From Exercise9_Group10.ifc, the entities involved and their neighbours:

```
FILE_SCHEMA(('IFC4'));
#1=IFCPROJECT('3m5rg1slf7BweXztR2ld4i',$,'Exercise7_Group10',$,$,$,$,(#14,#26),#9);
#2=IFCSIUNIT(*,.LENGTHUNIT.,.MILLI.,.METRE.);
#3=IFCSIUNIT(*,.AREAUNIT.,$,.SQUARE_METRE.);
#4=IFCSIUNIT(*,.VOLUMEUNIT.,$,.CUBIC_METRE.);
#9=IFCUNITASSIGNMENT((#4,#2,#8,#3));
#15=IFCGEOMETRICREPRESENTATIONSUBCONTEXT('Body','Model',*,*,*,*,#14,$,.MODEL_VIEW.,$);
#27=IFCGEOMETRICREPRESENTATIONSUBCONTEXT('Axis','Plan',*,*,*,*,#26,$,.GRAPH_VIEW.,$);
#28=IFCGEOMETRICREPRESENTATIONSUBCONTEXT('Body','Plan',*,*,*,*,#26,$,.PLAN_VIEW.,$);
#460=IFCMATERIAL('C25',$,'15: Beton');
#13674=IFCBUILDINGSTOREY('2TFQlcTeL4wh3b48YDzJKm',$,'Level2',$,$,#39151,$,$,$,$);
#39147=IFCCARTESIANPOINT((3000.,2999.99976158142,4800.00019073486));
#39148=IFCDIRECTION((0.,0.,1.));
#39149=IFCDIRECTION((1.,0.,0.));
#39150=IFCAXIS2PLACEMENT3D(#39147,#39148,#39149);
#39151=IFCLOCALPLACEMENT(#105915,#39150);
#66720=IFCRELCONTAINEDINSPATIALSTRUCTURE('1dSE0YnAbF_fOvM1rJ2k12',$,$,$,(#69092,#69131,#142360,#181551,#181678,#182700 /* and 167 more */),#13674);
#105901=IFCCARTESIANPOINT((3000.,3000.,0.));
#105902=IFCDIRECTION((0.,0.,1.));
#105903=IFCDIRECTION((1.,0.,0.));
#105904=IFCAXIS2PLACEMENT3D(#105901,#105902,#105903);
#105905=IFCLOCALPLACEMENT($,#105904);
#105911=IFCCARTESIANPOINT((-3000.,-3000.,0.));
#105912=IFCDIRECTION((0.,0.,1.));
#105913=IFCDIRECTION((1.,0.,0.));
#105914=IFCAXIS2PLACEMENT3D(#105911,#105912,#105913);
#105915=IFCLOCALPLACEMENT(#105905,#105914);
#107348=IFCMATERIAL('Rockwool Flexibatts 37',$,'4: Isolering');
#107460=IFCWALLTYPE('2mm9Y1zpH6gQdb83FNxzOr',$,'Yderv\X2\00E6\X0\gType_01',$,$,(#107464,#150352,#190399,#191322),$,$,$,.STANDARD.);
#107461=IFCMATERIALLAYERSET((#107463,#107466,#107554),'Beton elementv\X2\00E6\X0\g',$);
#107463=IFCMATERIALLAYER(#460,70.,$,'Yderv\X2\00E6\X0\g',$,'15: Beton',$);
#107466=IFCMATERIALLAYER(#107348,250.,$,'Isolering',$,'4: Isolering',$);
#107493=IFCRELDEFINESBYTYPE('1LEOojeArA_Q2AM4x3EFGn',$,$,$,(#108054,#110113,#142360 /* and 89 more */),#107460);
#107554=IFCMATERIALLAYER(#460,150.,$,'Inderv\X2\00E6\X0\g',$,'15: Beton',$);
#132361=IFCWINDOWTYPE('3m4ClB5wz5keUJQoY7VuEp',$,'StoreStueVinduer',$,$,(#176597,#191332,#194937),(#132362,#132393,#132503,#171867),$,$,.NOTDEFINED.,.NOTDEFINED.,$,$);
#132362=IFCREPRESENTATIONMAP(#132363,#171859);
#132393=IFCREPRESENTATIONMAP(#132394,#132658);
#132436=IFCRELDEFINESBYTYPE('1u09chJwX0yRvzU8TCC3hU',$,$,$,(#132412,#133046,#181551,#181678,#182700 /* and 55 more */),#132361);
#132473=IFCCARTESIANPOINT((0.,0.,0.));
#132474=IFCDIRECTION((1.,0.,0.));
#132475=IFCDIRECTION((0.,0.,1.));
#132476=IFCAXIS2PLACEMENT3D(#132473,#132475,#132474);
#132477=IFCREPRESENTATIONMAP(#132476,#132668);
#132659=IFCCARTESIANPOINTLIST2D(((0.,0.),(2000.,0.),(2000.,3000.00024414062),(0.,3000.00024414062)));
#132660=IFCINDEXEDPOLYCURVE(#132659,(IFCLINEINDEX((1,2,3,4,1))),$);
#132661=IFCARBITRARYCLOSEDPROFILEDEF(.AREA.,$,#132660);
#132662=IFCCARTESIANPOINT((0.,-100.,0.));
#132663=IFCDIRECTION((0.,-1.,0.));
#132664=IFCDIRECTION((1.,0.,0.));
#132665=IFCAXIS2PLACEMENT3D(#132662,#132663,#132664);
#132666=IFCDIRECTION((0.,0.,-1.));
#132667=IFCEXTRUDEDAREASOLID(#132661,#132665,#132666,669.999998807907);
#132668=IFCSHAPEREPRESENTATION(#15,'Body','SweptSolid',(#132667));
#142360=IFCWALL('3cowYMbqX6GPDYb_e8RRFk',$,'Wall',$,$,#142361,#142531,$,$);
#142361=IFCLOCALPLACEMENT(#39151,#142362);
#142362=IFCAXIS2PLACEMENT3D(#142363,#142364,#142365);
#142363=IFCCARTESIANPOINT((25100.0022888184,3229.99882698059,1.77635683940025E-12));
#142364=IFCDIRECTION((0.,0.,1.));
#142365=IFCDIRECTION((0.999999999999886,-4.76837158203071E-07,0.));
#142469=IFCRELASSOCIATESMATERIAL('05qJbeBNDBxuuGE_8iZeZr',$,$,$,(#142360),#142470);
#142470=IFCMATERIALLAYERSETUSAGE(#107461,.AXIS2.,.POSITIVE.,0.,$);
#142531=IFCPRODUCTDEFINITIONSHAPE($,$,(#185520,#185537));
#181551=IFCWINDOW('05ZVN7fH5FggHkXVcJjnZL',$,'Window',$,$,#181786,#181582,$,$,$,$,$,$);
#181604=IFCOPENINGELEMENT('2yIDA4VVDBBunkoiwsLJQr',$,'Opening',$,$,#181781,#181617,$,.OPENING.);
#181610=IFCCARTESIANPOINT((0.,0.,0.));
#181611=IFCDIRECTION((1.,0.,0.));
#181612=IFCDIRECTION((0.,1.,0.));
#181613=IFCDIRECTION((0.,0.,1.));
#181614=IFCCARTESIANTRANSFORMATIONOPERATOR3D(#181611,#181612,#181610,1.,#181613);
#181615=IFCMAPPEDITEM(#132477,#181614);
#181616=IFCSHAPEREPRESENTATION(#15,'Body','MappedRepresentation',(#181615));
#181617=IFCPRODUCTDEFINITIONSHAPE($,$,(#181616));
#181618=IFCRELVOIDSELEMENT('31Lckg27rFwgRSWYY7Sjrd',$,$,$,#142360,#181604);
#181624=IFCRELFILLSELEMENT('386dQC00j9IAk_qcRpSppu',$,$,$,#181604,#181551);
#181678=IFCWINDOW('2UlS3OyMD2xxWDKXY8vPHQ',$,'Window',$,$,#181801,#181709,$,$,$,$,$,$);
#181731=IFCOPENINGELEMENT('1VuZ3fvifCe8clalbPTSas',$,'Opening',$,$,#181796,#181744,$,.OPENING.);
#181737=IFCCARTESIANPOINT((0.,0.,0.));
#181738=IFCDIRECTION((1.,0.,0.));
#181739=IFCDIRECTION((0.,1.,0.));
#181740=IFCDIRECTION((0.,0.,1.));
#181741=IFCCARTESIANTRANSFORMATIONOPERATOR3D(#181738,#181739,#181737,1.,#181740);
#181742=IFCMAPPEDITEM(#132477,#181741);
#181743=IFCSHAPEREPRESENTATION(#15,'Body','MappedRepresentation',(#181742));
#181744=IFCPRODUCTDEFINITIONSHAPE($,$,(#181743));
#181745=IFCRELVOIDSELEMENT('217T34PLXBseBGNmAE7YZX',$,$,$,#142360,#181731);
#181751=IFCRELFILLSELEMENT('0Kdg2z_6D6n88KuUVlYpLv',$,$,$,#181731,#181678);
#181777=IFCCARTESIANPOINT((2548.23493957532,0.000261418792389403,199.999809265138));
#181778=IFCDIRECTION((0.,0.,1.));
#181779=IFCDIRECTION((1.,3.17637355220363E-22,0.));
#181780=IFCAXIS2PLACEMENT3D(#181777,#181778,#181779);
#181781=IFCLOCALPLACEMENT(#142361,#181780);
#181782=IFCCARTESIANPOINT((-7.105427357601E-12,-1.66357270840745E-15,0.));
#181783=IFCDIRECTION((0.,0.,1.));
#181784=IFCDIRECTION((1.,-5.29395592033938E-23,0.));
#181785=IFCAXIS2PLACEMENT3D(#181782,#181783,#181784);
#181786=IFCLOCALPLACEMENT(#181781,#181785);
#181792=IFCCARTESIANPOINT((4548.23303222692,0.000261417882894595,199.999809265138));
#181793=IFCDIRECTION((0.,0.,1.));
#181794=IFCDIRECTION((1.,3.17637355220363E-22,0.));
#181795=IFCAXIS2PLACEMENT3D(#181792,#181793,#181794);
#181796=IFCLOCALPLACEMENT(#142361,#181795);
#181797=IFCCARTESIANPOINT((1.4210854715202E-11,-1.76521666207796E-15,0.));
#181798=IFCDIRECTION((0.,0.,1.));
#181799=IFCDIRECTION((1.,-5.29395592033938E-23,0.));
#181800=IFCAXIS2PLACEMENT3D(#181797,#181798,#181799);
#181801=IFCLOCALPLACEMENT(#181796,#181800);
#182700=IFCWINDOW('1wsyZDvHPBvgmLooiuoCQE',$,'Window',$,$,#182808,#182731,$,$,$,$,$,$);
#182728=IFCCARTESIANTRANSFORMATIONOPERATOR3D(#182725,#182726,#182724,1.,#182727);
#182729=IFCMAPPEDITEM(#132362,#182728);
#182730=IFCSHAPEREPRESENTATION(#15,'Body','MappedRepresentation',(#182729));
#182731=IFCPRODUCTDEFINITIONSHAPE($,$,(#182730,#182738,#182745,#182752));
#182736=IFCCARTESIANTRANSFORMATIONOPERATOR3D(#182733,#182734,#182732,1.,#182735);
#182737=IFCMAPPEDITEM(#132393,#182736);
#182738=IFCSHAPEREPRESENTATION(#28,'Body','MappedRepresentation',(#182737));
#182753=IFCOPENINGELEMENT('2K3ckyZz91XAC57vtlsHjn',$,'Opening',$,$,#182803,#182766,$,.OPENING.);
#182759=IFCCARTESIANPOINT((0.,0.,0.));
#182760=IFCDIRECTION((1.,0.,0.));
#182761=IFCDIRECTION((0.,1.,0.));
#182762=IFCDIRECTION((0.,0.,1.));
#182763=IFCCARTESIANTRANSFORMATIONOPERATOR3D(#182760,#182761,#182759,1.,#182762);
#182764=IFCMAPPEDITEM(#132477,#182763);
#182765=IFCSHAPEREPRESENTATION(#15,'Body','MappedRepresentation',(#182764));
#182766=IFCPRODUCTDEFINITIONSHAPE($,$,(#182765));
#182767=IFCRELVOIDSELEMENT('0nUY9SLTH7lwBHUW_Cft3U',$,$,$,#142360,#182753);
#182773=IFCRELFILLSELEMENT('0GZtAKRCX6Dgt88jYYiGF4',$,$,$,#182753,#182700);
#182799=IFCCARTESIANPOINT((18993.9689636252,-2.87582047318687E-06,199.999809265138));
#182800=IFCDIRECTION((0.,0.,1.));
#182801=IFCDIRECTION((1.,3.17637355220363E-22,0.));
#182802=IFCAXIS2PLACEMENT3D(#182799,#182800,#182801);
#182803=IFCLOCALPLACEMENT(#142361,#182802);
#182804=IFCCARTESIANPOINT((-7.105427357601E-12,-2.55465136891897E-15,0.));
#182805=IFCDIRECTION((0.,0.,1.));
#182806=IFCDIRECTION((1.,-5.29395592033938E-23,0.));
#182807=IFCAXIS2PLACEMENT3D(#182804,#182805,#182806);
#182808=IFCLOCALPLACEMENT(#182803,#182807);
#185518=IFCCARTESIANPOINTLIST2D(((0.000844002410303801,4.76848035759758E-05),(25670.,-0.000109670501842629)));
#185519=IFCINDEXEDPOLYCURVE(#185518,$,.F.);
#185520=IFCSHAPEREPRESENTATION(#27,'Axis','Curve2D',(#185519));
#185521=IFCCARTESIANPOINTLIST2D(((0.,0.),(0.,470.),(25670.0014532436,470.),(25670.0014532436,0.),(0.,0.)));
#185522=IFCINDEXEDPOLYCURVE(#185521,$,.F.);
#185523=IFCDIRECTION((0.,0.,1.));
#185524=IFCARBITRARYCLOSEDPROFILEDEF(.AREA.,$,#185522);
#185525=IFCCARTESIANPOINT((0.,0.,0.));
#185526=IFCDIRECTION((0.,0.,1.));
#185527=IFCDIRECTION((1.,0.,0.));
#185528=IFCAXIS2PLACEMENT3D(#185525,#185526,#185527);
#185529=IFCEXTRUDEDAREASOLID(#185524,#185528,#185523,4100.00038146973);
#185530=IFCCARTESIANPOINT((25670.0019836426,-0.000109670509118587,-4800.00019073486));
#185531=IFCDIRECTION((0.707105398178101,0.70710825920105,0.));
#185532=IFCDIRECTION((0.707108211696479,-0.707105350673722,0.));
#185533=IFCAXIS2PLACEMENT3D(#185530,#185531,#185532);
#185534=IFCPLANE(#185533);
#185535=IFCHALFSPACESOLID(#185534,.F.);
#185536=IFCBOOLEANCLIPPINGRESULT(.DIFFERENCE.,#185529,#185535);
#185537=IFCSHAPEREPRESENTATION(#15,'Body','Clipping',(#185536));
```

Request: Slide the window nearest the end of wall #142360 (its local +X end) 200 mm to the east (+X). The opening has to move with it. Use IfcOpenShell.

```python
import ifcopenshell
import ifcopenshell.api.geometry
import ifcopenshell.util.placement
import ifcopenshell.util.unit

model = ifcopenshell.open("Exercise9_Group10.ifc")
unit_scale = ifcopenshell.util.unit.calculate_unit_scale(model)

window = model.by_guid("1wsyZDvHPBvgmLooiuoCQE")
opening = window.FillsVoids[0].RelatingOpeningElement
wall = opening.VoidsElements[0].RelatingBuildingElement

wall_matrix = ifcopenshell.util.placement.get_local_placement(wall.ObjectPlacement)
shift = wall_matrix[:3, 0] * 0.2 / unit_scale
before = ifcopenshell.util.placement.get_local_placement(window.ObjectPlacement)[:3, 3].copy()

# The window is placed relative to its opening, so it follows when the opening moves.
matrix = ifcopenshell.util.placement.get_local_placement(opening.ObjectPlacement)
matrix[:3, 3] += shift
ifcopenshell.api.geometry.edit_object_placement(
    model, product=opening, matrix=matrix, is_si=False, should_transform_children=True
)

after = ifcopenshell.util.placement.get_local_placement(window.ObjectPlacement)[:3, 3]
print("window moved by", (after - before).round(3) + 0.0)

model.write("Exercise9_Group10_edited.ifc")
```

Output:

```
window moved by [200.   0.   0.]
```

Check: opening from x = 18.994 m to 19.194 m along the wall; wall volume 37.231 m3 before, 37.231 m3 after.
